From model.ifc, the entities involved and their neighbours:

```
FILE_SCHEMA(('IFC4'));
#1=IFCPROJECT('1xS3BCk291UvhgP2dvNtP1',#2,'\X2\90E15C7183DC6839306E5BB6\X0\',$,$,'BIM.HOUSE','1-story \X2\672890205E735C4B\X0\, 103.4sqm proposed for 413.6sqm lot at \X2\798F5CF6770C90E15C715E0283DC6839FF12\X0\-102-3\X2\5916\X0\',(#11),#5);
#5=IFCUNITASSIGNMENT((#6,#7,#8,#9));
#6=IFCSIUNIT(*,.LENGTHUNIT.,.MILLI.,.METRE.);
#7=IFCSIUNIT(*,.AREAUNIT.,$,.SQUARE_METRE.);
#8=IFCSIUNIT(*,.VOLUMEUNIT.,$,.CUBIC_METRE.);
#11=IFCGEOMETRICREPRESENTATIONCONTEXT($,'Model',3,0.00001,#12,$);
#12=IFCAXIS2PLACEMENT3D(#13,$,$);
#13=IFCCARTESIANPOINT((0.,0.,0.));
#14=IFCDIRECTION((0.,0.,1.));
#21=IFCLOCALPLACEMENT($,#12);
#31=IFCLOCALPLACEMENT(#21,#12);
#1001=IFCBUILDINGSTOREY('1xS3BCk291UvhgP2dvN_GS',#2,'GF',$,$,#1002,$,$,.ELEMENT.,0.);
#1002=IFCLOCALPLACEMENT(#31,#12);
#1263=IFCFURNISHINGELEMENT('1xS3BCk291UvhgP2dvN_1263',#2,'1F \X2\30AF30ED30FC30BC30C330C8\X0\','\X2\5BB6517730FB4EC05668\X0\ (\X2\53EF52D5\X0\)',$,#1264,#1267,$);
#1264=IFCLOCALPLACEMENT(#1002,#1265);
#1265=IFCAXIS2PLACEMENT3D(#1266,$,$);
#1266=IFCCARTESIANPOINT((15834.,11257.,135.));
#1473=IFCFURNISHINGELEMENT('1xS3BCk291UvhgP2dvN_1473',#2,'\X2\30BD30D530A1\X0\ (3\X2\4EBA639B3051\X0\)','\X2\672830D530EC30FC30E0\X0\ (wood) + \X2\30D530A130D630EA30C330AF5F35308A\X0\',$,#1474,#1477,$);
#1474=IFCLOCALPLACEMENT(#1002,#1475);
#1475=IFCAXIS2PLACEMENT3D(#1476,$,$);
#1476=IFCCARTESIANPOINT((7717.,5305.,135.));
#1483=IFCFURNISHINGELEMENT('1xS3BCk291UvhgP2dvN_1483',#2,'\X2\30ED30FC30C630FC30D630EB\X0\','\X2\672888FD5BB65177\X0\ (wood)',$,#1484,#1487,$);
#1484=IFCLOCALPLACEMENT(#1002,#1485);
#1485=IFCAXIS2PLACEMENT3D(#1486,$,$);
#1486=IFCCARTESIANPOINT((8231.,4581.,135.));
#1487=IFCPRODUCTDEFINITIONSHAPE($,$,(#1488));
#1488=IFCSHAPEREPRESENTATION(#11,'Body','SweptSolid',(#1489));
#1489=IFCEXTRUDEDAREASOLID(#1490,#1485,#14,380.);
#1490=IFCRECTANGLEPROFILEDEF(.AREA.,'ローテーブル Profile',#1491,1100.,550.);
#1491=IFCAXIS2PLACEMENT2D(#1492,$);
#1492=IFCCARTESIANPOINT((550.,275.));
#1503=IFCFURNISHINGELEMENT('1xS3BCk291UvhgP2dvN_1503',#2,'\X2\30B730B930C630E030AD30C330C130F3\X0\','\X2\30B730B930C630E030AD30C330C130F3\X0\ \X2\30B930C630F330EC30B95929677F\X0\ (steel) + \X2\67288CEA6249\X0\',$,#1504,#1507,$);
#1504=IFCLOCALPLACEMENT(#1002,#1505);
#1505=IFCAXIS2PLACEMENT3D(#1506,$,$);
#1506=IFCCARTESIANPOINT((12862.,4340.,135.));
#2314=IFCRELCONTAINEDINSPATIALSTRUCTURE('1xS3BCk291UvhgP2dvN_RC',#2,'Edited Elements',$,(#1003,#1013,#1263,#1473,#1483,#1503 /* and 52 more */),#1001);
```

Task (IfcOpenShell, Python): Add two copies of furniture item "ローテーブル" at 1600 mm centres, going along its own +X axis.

```python
import ifcopenshell
import ifcopenshell.api.geometry
import ifcopenshell.api.root
import ifcopenshell.util.element
import ifcopenshell.util.placement
import ifcopenshell.util.unit

model = ifcopenshell.open("model.ifc")
unit_scale = ifcopenshell.util.unit.calculate_unit_scale(model)


def reuse_history(source, copy):
    """copy_class also copies each property set's owner history, people and application; keep the originals."""
    for rel in copy.IsDefinedBy:
        if rel.is_a("IfcRelDefinesByProperties") and (history := rel.RelatingPropertyDefinition.OwnerHistory):
            rel.RelatingPropertyDefinition.OwnerHistory = source.OwnerHistory
            ifcopenshell.util.element.remove_deep2(model, history)


source = model.by_guid("1xS3BCk291UvhgP2dvN_1483")
base = ifcopenshell.util.placement.get_local_placement(source.ObjectPlacement)
step = base[:3, 0] * 1.6 / unit_scale

for i in range(1, 3):
    copy = ifcopenshell.api.root.copy_class(model, product=source)
    copy.Representation = ifcopenshell.util.element.copy_deep(
        model, source.Representation, exclude=["IfcGeometricRepresentationContext", "IfcRepresentationMap"]
    )
    reuse_history(source, copy)
    matrix = base.copy()
    matrix[:3, 3] += i * step
    print("added at", matrix[:3, 3].round(3) + 0.0)
    ifcopenshell.api.geometry.edit_object_placement(model, product=copy, matrix=matrix, is_si=False)

model.write("model_updated.ifc")
```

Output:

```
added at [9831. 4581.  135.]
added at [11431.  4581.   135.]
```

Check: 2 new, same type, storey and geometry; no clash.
